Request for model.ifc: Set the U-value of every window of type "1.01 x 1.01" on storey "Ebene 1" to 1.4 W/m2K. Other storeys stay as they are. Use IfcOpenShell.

First a look at what the model holds.

```python
import ifcopenshell
import ifcopenshell.util.element

model = ifcopenshell.open("model.ifc")
print(model.schema)
storey = next(s for s in model.by_type("IfcBuildingStorey") if s.Name == "Ebene 1")
windows = [e for e in ifcopenshell.util.element.get_decomposition(storey) if e.is_a("IfcWindow")]
seen = {}
for e in windows:
    element_type = ifcopenshell.util.element.get_type(e)
    key = (element_type.Name if element_type != e and element_type else None, ifcopenshell.util.element.get_pset(e, "Pset_WindowCommon", "ThermalTransmittance"))
    seen[key] = seen.get(key, 0) + 1
for (name, value), count in sorted(seen.items(), key=str):
    print(count, "x", name, "|", value)
```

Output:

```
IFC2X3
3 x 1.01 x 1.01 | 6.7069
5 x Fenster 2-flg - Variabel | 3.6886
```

```python
import ifcopenshell
import ifcopenshell.api.pset
import ifcopenshell.util.element

model = ifcopenshell.open("model.ifc")

storey = next(s for s in model.by_type("IfcBuildingStorey") if s.Name == "Ebene 1")
windows = [e for e in ifcopenshell.util.element.get_decomposition(storey) if e.is_a("IfcWindow")]

count = 0
for e in windows:
    element_type = ifcopenshell.util.element.get_type(e)
    if element_type in (None, e) or element_type.Name != "1.01 x 1.01":
        continue
    # add_pset returns the element's existing set when there is one.
    pset = ifcopenshell.api.pset.add_pset(model, product=e, name="Pset_WindowCommon")
    ifcopenshell.api.pset.edit_pset(model, pset=pset, properties={"ThermalTransmittance": 1.4})
    count += 1

print(count, "windows updated")

model.write("model_edited.ifc")
```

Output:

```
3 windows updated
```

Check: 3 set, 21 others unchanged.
